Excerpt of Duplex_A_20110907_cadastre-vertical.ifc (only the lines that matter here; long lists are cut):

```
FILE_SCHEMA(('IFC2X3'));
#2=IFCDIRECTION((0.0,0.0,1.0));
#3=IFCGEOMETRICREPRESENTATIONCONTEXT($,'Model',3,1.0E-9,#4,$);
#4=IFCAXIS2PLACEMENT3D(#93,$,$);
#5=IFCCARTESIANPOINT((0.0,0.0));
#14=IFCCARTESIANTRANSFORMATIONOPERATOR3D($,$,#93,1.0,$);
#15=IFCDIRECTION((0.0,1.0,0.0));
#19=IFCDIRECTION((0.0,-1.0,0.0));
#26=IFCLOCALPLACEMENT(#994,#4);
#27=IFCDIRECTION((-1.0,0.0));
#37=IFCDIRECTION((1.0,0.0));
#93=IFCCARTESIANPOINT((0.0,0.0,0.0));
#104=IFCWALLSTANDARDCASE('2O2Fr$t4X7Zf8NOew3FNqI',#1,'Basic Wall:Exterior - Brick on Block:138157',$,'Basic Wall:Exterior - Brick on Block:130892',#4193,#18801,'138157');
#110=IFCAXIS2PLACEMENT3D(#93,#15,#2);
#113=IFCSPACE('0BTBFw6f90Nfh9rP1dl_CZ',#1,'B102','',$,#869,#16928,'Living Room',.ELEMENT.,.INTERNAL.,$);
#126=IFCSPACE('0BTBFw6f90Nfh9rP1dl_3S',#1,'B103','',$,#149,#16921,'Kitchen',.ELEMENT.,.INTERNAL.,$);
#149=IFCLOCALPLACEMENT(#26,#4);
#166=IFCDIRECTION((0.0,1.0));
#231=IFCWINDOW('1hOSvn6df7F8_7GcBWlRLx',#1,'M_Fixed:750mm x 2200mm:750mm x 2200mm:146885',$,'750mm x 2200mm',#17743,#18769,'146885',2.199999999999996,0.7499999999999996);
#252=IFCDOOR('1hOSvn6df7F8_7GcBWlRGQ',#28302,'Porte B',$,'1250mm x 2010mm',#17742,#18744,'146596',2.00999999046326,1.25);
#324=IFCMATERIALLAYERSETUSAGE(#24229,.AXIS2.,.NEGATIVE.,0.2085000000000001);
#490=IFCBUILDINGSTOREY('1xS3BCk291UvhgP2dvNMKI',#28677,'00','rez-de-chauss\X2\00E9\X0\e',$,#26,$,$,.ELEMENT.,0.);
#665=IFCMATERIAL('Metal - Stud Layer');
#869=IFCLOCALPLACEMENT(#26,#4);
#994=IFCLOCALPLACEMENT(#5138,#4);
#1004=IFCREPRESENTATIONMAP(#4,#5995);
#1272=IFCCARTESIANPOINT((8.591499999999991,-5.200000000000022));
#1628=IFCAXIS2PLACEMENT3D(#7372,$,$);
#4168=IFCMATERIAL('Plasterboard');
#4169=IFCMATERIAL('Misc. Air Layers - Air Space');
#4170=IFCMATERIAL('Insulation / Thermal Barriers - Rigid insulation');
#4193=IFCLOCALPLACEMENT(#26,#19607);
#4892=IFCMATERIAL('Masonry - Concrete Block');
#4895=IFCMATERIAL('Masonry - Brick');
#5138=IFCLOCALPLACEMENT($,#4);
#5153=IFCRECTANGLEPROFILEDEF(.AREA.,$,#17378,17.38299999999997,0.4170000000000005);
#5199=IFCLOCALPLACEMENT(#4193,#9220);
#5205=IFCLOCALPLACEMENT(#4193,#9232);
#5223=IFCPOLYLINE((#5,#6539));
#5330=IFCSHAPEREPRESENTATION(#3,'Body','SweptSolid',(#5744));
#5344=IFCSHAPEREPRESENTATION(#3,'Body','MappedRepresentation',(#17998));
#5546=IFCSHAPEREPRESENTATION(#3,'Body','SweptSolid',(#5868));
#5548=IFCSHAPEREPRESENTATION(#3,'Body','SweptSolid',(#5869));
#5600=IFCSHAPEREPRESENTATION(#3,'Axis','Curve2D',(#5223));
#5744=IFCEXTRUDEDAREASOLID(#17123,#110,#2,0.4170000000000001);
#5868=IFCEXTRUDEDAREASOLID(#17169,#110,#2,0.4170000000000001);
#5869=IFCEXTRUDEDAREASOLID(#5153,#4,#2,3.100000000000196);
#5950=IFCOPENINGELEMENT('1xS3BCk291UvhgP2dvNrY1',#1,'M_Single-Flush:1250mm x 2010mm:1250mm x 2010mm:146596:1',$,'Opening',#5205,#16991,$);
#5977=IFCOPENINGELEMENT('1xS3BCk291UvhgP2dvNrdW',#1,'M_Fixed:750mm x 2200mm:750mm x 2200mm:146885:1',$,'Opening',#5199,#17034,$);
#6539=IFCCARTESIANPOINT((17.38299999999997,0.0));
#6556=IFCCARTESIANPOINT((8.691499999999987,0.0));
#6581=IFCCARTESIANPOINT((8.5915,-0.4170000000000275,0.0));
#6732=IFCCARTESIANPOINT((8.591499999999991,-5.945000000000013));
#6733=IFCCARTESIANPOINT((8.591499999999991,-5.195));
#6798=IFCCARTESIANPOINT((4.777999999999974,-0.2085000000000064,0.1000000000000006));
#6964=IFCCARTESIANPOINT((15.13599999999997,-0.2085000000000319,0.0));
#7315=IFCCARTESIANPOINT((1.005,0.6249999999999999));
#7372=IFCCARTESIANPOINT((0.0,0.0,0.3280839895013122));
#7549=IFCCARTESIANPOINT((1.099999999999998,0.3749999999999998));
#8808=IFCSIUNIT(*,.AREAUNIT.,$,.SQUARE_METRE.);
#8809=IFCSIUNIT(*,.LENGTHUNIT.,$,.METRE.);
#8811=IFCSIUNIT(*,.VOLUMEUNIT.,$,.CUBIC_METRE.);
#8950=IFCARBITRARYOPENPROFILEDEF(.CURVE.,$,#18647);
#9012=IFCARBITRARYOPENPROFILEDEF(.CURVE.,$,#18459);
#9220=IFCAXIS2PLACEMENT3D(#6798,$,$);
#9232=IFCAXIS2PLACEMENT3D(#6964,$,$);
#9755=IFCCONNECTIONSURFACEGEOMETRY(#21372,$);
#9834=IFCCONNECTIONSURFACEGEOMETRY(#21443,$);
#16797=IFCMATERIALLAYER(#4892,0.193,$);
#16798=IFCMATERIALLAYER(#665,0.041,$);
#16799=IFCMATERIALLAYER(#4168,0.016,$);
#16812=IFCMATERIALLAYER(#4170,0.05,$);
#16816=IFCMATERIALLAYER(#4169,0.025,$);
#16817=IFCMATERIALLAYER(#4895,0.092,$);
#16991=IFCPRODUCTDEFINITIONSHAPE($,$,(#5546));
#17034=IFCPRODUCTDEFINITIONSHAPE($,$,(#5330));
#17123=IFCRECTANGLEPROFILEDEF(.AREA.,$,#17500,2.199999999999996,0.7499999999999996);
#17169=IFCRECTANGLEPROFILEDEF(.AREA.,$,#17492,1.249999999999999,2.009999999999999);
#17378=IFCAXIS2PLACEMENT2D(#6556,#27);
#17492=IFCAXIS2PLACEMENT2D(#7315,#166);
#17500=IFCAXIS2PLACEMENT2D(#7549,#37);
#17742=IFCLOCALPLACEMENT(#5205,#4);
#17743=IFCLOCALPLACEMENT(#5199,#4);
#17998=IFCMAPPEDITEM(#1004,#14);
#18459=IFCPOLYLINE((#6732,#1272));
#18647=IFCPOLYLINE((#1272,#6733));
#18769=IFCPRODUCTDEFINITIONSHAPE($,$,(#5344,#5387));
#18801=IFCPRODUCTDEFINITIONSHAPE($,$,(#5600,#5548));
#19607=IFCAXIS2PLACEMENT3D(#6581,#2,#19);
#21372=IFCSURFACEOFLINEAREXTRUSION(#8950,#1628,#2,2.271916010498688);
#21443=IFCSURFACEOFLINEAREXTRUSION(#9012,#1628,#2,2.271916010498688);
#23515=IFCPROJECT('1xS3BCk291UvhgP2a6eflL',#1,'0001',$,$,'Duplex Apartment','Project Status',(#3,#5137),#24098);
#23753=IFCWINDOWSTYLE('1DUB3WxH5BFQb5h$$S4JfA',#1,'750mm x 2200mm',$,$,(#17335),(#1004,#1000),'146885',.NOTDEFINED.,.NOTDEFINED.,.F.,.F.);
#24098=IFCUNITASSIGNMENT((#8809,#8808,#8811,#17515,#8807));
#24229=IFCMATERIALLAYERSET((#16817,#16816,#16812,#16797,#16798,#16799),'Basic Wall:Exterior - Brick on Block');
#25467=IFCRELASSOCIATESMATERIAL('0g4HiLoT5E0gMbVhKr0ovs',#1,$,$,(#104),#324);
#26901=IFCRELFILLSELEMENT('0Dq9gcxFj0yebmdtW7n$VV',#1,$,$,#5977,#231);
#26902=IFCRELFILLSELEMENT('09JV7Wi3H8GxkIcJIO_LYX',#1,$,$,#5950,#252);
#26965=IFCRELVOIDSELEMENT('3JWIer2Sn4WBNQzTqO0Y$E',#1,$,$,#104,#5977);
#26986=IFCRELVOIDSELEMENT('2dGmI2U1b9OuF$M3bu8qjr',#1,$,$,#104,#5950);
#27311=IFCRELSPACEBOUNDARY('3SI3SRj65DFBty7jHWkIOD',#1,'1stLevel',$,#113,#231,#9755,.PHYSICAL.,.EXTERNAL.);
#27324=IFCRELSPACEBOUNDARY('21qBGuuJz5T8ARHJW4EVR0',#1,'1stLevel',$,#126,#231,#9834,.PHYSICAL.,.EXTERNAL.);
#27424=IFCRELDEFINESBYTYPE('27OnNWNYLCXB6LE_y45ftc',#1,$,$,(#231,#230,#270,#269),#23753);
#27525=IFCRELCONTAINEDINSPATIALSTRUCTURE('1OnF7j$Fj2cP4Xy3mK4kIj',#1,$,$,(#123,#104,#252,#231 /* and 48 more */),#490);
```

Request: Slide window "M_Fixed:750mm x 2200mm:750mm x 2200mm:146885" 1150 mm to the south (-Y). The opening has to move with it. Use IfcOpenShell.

```python
import numpy as np
import ifcopenshell
import ifcopenshell.api.geometry
import ifcopenshell.util.placement
import ifcopenshell.util.unit

model = ifcopenshell.open("Duplex_A_20110907_cadastre-vertical.ifc")
unit_scale = ifcopenshell.util.unit.calculate_unit_scale(model)

window = model.by_guid("1hOSvn6df7F8_7GcBWlRLx")
opening = window.FillsVoids[0].RelatingOpeningElement
wall = opening.VoidsElements[0].RelatingBuildingElement

wall_matrix = ifcopenshell.util.placement.get_local_placement(wall.ObjectPlacement)
shift = wall_matrix[:3, 0] * 1.15 / unit_scale
before = ifcopenshell.util.placement.get_local_placement(window.ObjectPlacement)[:3, 3].copy()

# The window is placed relative to its opening, so it follows when the opening moves.
matrix = ifcopenshell.util.placement.get_local_placement(opening.ObjectPlacement)
matrix[:3, 3] += shift
ifcopenshell.api.geometry.edit_object_placement(
    model, product=opening, matrix=matrix, is_si=False, should_transform_children=True
)

# Space boundary surfaces are stored in each space's coordinates; move them too.
for rel in window.ProvidesBoundaries:
    if not rel.ConnectionGeometry:
        continue
    surface = rel.ConnectionGeometry.SurfaceOnRelatingElement
    space_matrix = ifcopenshell.util.placement.get_local_placement(rel.RelatingSpace.ObjectPlacement)
    point = np.array(surface.Position.Location.Coordinates) + space_matrix[:3, :3].T @ shift
    surface.Position = model.createIfcAxis2Placement3D(
        model.createIfcCartesianPoint(point.tolist()), surface.Position.Axis, surface.Position.RefDirection
    )

after = ifcopenshell.util.placement.get_local_placement(window.ObjectPlacement)[:3, 3]
print("window moved by", (after - before).round(3) + 0.0)

model.write("Duplex_A_20110907_cadastre-vertical_rev.ifc")
```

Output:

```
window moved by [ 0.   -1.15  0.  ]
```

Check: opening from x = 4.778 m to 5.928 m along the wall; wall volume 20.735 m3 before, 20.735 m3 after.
